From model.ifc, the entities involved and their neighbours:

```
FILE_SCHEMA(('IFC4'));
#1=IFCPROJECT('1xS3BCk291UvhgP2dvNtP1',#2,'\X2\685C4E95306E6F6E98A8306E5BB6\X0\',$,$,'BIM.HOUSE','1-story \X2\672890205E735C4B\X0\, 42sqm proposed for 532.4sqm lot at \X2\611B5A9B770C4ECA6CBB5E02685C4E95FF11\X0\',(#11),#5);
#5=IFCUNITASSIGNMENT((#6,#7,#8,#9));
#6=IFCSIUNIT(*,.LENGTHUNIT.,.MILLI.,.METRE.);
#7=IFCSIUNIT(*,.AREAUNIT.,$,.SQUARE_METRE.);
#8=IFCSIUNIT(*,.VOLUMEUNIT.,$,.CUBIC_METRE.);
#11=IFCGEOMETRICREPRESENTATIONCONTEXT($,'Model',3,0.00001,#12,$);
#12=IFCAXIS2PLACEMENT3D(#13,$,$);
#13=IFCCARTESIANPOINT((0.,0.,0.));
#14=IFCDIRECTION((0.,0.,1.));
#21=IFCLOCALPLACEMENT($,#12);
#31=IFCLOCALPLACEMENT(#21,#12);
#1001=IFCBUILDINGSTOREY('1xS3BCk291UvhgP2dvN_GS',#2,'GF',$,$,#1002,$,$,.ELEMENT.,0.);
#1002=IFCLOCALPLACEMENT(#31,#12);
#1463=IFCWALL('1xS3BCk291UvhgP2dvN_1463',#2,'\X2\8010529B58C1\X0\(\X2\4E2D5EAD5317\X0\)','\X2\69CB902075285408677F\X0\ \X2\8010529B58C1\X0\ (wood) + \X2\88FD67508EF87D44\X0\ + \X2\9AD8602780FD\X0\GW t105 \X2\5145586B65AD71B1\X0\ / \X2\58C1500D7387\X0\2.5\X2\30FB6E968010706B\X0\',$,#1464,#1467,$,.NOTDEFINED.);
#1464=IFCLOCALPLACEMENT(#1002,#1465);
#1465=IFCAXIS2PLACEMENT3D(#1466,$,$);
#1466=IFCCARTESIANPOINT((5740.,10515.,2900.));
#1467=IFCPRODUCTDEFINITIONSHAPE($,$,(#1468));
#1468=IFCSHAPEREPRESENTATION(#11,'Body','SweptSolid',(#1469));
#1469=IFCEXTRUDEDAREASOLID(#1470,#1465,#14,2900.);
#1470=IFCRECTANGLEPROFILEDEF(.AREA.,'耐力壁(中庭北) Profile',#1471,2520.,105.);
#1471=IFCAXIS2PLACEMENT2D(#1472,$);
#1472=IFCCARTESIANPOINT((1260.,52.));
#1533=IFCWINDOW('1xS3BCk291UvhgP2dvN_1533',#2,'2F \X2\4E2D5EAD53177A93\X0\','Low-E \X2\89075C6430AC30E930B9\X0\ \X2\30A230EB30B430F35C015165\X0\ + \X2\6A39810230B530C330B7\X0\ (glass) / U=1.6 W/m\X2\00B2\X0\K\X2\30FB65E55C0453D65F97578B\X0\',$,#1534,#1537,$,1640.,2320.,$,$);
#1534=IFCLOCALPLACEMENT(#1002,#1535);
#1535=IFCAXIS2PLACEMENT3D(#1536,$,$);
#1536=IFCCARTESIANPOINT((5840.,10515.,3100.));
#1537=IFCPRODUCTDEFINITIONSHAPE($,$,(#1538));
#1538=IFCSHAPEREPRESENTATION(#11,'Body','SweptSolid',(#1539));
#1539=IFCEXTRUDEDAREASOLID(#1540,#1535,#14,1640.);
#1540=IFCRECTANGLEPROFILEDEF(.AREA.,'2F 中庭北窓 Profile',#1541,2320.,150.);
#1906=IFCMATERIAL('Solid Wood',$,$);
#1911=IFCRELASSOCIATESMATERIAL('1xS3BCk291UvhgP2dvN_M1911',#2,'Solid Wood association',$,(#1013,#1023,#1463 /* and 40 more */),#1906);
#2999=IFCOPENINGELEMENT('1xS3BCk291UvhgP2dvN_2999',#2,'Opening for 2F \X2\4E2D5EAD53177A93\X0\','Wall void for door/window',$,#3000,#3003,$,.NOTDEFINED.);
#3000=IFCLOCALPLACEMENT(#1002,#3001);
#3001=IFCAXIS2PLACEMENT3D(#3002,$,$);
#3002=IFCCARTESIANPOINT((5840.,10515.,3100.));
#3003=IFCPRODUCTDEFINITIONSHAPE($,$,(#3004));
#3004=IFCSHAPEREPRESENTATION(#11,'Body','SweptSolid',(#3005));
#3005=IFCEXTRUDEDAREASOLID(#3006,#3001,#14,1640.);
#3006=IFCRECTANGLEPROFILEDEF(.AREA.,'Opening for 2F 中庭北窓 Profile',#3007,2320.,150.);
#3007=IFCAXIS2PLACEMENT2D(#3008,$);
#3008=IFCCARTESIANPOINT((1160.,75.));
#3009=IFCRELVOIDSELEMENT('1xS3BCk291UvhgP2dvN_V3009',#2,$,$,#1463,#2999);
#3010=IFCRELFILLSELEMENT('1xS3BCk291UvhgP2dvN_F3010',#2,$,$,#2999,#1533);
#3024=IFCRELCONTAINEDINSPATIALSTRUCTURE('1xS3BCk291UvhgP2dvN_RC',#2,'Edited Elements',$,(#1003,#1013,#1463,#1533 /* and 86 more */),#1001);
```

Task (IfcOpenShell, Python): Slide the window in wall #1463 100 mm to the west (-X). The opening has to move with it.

```python
import ifcopenshell
import ifcopenshell.api.geometry
import ifcopenshell.util.placement
import ifcopenshell.util.unit

model = ifcopenshell.open("model.ifc")
unit_scale = ifcopenshell.util.unit.calculate_unit_scale(model)

window = model.by_guid("1xS3BCk291UvhgP2dvN_1533")
opening = window.FillsVoids[0].RelatingOpeningElement
wall = opening.VoidsElements[0].RelatingBuildingElement

wall_matrix = ifcopenshell.util.placement.get_local_placement(wall.ObjectPlacement)
shift = wall_matrix[:3, 0] * -0.1 / unit_scale
before = ifcopenshell.util.placement.get_local_placement(window.ObjectPlacement)[:3, 3].copy()

# The window is not placed relative to its opening, so move both.
for product in (opening, window):
    matrix = ifcopenshell.util.placement.get_local_placement(product.ObjectPlacement)
    matrix[:3, 3] += shift
    ifcopenshell.api.geometry.edit_object_placement(model, product=product, matrix=matrix, is_si=False)

after = ifcopenshell.util.placement.get_local_placement(window.ObjectPlacement)[:3, 3]
print("window moved by", (after - before).round(3) + 0.0)

model.write("model_v2.ifc")
```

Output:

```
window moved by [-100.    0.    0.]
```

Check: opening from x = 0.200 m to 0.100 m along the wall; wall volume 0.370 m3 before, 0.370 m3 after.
